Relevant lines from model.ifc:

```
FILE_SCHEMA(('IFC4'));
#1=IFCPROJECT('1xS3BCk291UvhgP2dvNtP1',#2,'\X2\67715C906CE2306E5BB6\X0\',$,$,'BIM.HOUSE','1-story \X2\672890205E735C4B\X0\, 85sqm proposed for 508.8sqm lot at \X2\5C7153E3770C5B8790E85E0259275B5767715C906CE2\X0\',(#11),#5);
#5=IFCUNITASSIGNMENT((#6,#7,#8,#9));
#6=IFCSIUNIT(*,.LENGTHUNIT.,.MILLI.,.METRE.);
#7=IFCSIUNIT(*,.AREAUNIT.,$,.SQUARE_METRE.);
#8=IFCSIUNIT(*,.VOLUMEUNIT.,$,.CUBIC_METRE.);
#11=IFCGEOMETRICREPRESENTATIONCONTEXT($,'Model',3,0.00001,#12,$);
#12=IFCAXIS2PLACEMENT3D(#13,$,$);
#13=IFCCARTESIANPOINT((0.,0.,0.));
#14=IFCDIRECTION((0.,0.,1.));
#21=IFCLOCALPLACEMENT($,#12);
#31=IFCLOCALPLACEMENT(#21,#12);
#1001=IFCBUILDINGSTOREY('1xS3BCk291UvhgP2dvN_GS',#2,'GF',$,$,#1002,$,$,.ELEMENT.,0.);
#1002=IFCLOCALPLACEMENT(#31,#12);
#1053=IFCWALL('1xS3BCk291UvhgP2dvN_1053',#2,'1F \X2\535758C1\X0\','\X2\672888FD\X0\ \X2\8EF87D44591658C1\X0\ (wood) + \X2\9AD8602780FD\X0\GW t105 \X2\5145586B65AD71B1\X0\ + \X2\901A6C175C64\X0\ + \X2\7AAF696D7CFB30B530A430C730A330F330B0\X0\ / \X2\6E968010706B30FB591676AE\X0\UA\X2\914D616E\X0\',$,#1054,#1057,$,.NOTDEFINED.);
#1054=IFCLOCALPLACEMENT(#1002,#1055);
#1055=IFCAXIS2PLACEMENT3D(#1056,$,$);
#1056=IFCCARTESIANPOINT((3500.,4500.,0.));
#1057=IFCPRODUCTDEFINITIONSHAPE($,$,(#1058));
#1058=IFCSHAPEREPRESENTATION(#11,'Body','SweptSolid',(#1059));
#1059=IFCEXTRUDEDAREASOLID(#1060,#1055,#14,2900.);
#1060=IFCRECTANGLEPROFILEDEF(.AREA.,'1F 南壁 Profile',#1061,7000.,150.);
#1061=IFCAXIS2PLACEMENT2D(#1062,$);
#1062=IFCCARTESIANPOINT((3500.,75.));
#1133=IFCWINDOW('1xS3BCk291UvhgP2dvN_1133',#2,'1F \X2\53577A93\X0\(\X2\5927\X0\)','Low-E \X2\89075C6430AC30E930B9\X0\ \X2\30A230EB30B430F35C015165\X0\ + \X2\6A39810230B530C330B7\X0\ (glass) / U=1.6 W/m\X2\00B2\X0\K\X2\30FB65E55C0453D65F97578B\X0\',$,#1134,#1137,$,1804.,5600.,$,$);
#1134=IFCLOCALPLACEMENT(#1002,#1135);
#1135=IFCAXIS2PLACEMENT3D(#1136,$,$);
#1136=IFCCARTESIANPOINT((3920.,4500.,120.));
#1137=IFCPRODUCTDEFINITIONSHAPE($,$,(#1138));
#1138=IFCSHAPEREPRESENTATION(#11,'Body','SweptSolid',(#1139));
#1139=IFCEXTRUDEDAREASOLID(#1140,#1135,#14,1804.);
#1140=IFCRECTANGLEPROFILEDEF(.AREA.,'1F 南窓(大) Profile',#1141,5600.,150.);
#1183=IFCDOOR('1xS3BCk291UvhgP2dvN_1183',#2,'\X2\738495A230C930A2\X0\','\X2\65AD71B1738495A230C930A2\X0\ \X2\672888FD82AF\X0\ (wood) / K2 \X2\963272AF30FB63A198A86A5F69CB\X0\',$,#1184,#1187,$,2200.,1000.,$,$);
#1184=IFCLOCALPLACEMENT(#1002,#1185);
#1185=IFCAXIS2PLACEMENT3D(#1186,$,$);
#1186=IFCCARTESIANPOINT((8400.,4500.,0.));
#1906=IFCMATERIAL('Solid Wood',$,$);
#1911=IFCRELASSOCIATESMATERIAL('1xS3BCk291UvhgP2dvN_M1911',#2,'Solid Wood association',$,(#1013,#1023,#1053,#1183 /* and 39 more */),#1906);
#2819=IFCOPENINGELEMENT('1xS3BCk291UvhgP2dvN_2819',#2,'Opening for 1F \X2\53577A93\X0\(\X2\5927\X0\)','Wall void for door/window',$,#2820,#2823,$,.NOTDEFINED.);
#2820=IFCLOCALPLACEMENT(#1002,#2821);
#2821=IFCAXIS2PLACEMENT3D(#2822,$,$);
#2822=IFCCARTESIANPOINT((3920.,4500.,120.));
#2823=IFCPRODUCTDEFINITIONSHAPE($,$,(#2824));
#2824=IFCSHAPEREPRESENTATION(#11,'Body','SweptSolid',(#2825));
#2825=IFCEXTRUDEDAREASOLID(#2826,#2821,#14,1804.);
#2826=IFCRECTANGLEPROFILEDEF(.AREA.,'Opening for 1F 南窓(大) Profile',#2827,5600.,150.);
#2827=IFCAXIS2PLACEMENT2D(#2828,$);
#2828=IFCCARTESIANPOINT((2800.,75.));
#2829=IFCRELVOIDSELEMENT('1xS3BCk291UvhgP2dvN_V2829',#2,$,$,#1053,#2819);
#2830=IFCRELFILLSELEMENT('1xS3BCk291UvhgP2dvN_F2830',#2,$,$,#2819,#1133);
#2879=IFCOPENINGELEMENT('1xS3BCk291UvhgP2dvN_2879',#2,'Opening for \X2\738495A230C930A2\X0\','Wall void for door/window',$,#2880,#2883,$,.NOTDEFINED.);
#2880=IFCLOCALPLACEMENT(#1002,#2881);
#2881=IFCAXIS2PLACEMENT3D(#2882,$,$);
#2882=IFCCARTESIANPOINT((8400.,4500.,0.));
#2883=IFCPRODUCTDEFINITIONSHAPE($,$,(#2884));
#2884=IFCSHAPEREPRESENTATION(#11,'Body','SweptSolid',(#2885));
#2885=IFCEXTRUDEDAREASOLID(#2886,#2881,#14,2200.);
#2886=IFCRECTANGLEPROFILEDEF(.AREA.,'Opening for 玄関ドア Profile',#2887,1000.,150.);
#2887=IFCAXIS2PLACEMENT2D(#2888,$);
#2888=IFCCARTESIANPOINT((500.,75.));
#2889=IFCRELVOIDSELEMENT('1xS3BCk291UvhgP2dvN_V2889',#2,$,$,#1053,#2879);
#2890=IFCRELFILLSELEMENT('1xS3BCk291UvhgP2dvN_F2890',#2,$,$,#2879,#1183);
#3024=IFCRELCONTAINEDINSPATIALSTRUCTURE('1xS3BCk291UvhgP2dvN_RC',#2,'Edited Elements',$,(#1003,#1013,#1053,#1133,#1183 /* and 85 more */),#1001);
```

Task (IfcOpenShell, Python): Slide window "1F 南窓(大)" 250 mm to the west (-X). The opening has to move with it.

```python
import ifcopenshell
import ifcopenshell.api.geometry
import ifcopenshell.util.placement
import ifcopenshell.util.unit

model = ifcopenshell.open("model.ifc")
unit_scale = ifcopenshell.util.unit.calculate_unit_scale(model)

window = model.by_guid("1xS3BCk291UvhgP2dvN_1133")
opening = window.FillsVoids[0].RelatingOpeningElement
wall = opening.VoidsElements[0].RelatingBuildingElement

wall_matrix = ifcopenshell.util.placement.get_local_placement(wall.ObjectPlacement)
shift = wall_matrix[:3, 0] * -0.25 / unit_scale
before = ifcopenshell.util.placement.get_local_placement(window.ObjectPlacement)[:3, 3].copy()

# The window is not placed relative to its opening, so move both.
for product in (opening, window):
    matrix = ifcopenshell.util.placement.get_local_placement(product.ObjectPlacement)
    matrix[:3, 3] += shift
    ifcopenshell.api.geometry.edit_object_placement(model, product=product, matrix=matrix, is_si=False)

after = ifcopenshell.util.placement.get_local_placement(window.ObjectPlacement)[:3, 3]
print("window moved by", (after - before).round(3) + 0.0)

model.write("model_v2.ifc")
```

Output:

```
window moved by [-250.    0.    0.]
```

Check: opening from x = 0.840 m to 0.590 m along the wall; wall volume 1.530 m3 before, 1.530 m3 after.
